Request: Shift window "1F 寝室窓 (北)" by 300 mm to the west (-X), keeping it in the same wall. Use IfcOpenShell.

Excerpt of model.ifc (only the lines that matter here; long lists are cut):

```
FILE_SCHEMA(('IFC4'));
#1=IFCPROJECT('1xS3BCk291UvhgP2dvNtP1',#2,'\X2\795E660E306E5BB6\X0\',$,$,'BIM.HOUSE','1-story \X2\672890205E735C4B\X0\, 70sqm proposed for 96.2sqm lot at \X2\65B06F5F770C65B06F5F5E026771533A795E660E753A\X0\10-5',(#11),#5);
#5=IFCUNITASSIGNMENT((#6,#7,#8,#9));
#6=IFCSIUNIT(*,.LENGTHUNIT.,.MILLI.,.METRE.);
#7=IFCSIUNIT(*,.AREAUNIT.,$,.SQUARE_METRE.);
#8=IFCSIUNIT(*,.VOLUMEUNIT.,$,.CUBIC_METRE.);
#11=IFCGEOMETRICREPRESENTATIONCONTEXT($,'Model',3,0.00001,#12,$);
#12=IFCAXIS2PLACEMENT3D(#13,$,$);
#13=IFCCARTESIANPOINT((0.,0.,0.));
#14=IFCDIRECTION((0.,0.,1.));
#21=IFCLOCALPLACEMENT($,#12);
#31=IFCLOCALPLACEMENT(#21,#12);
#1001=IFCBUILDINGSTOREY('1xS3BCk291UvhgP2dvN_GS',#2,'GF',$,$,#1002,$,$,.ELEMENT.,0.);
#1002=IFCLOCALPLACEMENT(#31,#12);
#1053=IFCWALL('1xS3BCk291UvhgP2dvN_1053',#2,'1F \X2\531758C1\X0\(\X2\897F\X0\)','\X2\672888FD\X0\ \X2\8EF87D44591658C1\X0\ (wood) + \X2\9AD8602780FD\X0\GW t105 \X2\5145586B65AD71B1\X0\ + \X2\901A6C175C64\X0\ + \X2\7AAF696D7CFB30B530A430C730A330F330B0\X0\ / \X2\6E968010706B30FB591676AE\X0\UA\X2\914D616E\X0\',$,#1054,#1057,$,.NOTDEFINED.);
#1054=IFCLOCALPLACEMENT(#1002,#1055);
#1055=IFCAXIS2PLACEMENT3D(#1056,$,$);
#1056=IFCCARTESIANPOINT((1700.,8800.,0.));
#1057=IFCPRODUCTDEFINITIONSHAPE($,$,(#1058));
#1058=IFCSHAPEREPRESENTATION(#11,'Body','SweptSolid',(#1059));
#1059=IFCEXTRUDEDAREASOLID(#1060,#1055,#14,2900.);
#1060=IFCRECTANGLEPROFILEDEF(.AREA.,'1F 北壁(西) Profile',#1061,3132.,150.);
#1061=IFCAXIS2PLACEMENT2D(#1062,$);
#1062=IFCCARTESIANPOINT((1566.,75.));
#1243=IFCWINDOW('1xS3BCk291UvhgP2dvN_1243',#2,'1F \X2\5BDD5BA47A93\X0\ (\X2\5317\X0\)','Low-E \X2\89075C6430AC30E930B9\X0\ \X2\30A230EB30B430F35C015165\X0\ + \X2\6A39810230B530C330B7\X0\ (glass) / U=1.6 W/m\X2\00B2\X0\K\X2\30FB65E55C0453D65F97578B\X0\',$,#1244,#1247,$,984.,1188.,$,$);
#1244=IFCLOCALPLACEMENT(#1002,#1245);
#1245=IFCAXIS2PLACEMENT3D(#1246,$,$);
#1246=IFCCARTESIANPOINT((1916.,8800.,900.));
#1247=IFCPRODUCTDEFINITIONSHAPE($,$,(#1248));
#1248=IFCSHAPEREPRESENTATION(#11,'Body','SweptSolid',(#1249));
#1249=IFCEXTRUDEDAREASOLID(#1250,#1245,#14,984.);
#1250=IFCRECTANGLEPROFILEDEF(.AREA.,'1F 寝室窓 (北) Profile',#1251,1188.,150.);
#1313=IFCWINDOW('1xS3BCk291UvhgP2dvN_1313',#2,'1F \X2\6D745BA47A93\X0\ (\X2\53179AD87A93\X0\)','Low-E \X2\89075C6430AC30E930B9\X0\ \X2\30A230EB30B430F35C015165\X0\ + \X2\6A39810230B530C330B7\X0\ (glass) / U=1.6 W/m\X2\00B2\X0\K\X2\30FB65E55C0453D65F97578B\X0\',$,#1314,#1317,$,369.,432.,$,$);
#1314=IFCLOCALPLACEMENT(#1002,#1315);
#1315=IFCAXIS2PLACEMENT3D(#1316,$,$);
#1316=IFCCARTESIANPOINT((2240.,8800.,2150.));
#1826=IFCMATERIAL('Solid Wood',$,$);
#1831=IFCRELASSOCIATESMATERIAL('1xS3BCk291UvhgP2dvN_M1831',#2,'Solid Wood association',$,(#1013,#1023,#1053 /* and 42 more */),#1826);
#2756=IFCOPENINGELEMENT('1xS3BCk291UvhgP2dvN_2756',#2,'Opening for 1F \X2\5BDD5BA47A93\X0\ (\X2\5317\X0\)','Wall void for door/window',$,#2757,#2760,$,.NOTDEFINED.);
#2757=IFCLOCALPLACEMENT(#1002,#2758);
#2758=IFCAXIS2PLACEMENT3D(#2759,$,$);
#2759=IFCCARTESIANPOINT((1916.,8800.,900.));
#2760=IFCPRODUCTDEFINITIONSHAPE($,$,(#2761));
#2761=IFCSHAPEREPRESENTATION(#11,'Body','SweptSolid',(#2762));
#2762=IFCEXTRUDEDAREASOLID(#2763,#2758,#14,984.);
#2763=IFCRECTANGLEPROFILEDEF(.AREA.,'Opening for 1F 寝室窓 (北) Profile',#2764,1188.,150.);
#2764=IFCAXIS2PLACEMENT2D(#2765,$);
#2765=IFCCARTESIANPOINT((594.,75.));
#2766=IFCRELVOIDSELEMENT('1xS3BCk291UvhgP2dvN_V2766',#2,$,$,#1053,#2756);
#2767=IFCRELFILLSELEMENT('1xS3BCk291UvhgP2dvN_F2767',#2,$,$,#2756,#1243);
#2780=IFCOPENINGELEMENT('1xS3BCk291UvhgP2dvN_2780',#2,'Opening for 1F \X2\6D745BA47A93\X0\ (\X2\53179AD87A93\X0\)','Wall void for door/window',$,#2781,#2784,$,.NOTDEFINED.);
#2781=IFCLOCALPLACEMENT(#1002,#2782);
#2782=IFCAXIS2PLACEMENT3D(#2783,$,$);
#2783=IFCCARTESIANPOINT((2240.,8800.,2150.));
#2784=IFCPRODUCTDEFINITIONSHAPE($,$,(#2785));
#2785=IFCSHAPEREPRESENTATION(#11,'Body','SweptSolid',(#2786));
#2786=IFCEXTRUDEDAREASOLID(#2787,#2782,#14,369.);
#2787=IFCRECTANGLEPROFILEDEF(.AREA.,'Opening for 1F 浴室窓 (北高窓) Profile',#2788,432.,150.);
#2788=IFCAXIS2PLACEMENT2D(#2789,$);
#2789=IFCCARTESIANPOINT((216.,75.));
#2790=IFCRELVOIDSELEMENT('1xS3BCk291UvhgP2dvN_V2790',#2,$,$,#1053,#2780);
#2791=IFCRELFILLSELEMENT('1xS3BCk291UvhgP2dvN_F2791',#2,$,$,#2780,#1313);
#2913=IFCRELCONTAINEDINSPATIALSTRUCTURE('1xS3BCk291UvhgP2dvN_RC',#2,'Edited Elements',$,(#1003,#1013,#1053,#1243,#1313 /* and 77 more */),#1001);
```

```python
import ifcopenshell
import ifcopenshell.api.geometry
import ifcopenshell.util.placement
import ifcopenshell.util.unit

model = ifcopenshell.open("model.ifc")
unit_scale = ifcopenshell.util.unit.calculate_unit_scale(model)

window = model.by_guid("1xS3BCk291UvhgP2dvN_1243")
opening = window.FillsVoids[0].RelatingOpeningElement
wall = opening.VoidsElements[0].RelatingBuildingElement

wall_matrix = ifcopenshell.util.placement.get_local_placement(wall.ObjectPlacement)
shift = wall_matrix[:3, 0] * -0.3 / unit_scale
before = ifcopenshell.util.placement.get_local_placement(window.ObjectPlacement)[:3, 3].copy()

# The window is not placed relative to its opening, so move both.
for product in (opening, window):
    matrix = ifcopenshell.util.placement.get_local_placement(product.ObjectPlacement)
    matrix[:3, 3] += shift
    ifcopenshell.api.geometry.edit_object_placement(model, product=product, matrix=matrix, is_si=False)

after = ifcopenshell.util.placement.get_local_placement(window.ObjectPlacement)[:3, 3]
print("window moved by", (after - before).round(3) + 0.0)

model.write("model_rev.ifc")
```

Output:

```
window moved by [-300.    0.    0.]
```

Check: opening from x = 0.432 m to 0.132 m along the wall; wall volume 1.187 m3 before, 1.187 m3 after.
